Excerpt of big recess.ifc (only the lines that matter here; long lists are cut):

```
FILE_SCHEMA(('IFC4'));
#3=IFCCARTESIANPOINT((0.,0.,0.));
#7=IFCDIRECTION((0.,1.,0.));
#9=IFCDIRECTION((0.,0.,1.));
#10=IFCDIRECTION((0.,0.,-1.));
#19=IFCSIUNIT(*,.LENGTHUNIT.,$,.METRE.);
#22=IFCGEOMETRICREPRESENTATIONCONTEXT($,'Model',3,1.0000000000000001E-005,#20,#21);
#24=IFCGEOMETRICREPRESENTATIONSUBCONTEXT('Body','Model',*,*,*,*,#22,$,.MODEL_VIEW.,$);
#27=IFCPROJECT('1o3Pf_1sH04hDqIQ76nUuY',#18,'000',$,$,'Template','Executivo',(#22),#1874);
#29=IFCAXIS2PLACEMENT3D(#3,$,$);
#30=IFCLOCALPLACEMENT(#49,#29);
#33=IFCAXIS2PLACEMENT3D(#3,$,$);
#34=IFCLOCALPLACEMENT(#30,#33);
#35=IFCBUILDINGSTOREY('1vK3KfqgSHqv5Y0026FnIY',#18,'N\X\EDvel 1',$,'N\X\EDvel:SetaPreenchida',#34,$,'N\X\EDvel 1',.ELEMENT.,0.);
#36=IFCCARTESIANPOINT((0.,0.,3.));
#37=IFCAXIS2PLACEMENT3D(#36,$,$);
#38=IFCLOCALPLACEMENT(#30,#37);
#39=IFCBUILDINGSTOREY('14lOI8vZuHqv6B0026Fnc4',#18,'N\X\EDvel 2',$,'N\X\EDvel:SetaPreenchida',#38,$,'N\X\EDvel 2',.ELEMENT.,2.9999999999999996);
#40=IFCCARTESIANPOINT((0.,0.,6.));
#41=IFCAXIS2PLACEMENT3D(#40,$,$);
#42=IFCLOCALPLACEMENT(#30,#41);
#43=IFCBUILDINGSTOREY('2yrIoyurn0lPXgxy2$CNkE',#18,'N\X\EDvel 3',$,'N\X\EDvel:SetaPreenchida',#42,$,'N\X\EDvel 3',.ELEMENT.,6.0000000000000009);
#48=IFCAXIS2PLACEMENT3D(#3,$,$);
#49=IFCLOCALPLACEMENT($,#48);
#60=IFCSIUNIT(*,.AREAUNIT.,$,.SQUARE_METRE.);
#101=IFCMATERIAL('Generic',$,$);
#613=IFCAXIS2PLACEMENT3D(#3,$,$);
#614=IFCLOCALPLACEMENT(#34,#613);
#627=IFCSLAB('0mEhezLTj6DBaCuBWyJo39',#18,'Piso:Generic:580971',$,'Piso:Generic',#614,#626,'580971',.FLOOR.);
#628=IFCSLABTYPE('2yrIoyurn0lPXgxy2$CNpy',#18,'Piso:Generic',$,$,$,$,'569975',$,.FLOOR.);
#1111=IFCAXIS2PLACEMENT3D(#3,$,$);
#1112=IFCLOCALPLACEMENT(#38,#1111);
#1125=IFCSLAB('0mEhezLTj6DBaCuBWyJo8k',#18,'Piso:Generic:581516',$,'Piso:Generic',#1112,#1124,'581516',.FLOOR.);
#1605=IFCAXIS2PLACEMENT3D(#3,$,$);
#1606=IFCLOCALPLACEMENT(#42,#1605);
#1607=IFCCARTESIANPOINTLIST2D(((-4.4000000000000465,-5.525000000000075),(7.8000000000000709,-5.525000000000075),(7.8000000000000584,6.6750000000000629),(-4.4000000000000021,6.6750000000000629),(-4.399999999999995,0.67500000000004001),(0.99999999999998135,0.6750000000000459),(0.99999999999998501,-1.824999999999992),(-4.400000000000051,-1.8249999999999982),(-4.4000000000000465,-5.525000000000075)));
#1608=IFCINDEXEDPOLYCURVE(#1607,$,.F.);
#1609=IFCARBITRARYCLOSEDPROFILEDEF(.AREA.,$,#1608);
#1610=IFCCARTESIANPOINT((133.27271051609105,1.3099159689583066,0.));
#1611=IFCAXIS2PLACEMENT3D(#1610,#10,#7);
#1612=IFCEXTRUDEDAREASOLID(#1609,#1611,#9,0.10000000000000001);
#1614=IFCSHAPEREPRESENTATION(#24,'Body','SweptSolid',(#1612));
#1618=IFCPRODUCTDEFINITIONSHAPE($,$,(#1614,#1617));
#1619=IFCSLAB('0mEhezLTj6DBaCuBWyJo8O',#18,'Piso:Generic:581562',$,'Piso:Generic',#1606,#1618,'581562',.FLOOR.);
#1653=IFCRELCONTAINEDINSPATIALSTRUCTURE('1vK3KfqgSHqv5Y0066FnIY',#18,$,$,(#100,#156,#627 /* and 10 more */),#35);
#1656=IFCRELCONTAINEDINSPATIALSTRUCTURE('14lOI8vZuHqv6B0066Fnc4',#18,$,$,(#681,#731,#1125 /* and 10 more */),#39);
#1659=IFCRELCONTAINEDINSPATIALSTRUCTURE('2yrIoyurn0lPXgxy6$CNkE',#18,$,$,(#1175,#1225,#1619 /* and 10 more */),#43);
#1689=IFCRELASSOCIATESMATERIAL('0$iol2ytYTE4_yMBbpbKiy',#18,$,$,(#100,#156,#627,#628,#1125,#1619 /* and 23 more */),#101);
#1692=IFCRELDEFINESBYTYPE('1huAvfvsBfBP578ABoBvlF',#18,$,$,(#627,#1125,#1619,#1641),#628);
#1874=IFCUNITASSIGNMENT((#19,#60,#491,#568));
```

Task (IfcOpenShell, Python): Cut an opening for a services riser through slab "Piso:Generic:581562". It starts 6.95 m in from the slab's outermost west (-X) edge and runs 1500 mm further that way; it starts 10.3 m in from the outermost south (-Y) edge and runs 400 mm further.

```python
import numpy as np
import ifcopenshell
import ifcopenshell.api.feature
import ifcopenshell.api.geometry
import ifcopenshell.api.root
import ifcopenshell.geom
import ifcopenshell.util.placement
import ifcopenshell.util.representation
import ifcopenshell.util.shape
import ifcopenshell.util.unit

model = ifcopenshell.open("big recess.ifc")
unit_scale = ifcopenshell.util.unit.calculate_unit_scale(model)
settings = ifcopenshell.geom.settings()


def volume(element):
    """Net volume in cubic metres, openings subtracted."""
    shape = ifcopenshell.geom.create_shape(settings, element)
    return ifcopenshell.util.shape.get_volume(shape.geometry)


slab = model.by_id(1619)
before = volume(slab)

# Extent in the slab's own axes, in metres. The edges named are its -X and -Y sides.
slab_shape = ifcopenshell.geom.create_shape(settings, slab)
vertices = ifcopenshell.util.shape.get_vertices(slab_shape.geometry)
x_min, y_min, bottom = vertices.min(axis=0)
top = vertices[:, 2].max()

opening = ifcopenshell.api.root.create_entity(model, ifc_class="IfcOpeningElement", name="Services riser opening", predefined_type="OPENING")
context = ifcopenshell.util.representation.get_context(model, "Model", "Body", "MODEL_VIEW")
width, depth = 1.5, 0.4
outline = [(0.0, 0.0), (width, 0.0), (width, depth), (0.0, depth), (0.0, 0.0)]
# Overshoot both faces by 50 mm so the cut is clean.
shape = ifcopenshell.api.geometry.add_slab_representation(
    model, context=context, depth=top - bottom + 0.1, polyline=outline
)
ifcopenshell.api.geometry.assign_representation(model, product=opening, representation=shape)

matrix = ifcopenshell.util.placement.get_local_placement(slab.ObjectPlacement)
matrix[:, 3] = matrix @ np.append(np.array([x_min + 6.95, y_min + 10.3, bottom - 0.05]) / unit_scale, 1.0)
ifcopenshell.api.geometry.edit_object_placement(model, product=opening, matrix=matrix, is_si=False)
ifcopenshell.api.feature.add_feature(model, feature=opening, element=slab)

after = volume(slab)

print(f"slab volume {before:.3f} -> {after:.3f} m3")

model.write("big recess-out.ifc")
```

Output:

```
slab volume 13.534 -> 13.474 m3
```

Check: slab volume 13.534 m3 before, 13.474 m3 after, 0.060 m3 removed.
